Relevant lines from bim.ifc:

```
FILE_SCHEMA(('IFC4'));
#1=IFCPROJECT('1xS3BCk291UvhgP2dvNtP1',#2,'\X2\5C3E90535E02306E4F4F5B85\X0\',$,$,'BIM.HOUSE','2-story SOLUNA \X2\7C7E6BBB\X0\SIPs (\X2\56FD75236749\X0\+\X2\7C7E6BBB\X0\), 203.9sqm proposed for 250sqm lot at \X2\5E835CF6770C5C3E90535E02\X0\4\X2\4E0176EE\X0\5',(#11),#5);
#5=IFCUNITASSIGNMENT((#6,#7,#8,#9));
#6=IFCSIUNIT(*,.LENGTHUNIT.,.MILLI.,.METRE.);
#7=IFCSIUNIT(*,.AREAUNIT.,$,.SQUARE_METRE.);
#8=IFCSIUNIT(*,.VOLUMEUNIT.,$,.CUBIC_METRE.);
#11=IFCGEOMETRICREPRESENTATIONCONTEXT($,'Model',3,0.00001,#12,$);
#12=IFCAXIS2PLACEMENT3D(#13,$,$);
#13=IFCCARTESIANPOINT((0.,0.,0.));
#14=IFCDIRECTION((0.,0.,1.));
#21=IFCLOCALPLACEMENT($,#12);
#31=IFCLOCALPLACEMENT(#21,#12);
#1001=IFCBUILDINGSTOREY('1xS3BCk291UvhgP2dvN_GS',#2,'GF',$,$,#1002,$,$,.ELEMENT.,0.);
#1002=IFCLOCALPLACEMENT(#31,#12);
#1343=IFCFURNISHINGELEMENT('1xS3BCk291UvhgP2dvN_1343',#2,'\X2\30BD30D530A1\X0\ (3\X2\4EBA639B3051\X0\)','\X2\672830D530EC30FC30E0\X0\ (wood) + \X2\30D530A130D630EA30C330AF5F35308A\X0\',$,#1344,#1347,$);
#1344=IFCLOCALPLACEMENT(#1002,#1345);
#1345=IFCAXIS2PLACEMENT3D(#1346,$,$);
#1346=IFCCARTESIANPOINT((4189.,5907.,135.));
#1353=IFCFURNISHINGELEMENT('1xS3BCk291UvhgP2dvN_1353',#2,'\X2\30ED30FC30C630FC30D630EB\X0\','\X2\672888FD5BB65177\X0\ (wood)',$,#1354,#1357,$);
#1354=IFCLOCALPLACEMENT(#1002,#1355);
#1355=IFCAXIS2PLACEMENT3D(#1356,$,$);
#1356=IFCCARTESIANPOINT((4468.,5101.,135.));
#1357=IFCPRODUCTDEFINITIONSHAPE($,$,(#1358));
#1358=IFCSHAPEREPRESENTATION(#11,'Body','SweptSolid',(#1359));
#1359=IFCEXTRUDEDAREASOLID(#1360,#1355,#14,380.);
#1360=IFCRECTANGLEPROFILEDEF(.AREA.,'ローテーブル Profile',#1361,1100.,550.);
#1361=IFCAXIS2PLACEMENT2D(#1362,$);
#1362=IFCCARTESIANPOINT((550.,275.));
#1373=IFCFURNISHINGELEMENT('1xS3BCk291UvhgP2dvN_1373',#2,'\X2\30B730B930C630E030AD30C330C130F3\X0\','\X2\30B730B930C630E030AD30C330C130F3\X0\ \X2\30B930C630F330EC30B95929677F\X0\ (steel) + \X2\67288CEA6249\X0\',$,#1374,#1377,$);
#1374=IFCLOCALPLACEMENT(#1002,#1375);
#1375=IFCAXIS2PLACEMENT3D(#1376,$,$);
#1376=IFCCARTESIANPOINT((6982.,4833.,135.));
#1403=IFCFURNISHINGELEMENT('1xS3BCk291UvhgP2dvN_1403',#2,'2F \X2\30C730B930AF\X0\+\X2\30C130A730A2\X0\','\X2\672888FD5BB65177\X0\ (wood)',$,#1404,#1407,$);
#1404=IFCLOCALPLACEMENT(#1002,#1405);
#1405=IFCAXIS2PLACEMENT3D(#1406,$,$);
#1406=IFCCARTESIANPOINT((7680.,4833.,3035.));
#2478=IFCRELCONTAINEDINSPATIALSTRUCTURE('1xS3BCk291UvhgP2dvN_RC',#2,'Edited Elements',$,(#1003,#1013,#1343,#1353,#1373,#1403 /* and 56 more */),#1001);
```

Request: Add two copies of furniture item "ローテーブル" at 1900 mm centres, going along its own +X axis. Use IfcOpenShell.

```python
import ifcopenshell
import ifcopenshell.api.geometry
import ifcopenshell.api.root
import ifcopenshell.util.element
import ifcopenshell.util.placement
import ifcopenshell.util.unit

model = ifcopenshell.open("bim.ifc")
unit_scale = ifcopenshell.util.unit.calculate_unit_scale(model)


def reuse_history(source, copy):
    """copy_class also copies each property set's owner history, people and application; keep the originals."""
    for rel in copy.IsDefinedBy:
        if rel.is_a("IfcRelDefinesByProperties") and (history := rel.RelatingPropertyDefinition.OwnerHistory):
            rel.RelatingPropertyDefinition.OwnerHistory = source.OwnerHistory
            ifcopenshell.util.element.remove_deep2(model, history)


source = model.by_guid("1xS3BCk291UvhgP2dvN_1353")
base = ifcopenshell.util.placement.get_local_placement(source.ObjectPlacement)
step = base[:3, 0] * 1.9 / unit_scale

for i in range(1, 3):
    copy = ifcopenshell.api.root.copy_class(model, product=source)
    copy.Representation = ifcopenshell.util.element.copy_deep(
        model, source.Representation, exclude=["IfcGeometricRepresentationContext", "IfcRepresentationMap"]
    )
    reuse_history(source, copy)
    matrix = base.copy()
    matrix[:3, 3] += i * step
    print("added at", matrix[:3, 3].round(3) + 0.0)
    ifcopenshell.api.geometry.edit_object_placement(model, product=copy, matrix=matrix, is_si=False)

model.write("bim-out.ifc")
```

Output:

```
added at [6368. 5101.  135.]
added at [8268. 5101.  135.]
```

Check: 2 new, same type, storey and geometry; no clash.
